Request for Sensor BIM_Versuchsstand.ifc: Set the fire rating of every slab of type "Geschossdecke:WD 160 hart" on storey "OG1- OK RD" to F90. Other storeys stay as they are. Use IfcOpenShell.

First a look at what the model holds.

```python
import ifcopenshell
import ifcopenshell.util.element

model = ifcopenshell.open("Sensor BIM_Versuchsstand.ifc")
print(model.schema)
storey = next(s for s in model.by_type("IfcBuildingStorey") if s.Name == "OG1- OK RD")
slabs = [e for e in ifcopenshell.util.element.get_decomposition(storey) if e.is_a("IfcSlab")]
seen = {}
for e in slabs:
    element_type = ifcopenshell.util.element.get_type(e)
    key = (element_type.Name if element_type != e and element_type else None, ifcopenshell.util.element.get_pset(e, "Pset_SlabCommon", "FireRating"))
    seen[key] = seen.get(key, 0) + 1
for (name, value), count in sorted(seen.items(), key=str):
    print(count, "x", name, "|", value)
```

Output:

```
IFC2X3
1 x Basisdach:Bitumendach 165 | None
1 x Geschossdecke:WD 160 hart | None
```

```python
import ifcopenshell
import ifcopenshell.api.pset
import ifcopenshell.util.element

model = ifcopenshell.open("Sensor BIM_Versuchsstand.ifc")

storey = next(s for s in model.by_type("IfcBuildingStorey") if s.Name == "OG1- OK RD")
slabs = [e for e in ifcopenshell.util.element.get_decomposition(storey) if e.is_a("IfcSlab")]

count = 0
for e in slabs:
    element_type = ifcopenshell.util.element.get_type(e)
    if element_type in (None, e) or element_type.Name != "Geschossdecke:WD 160 hart":
        continue
    # add_pset returns the element's existing set when there is one.
    pset = ifcopenshell.api.pset.add_pset(model, product=e, name="Pset_SlabCommon")
    ifcopenshell.api.pset.edit_pset(model, pset=pset, properties={"FireRating": "F90"})
    count += 1

print(count, "slabs updated")

model.write("Sensor BIM_Versuchsstand_updated.ifc")
```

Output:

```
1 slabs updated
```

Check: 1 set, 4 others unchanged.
